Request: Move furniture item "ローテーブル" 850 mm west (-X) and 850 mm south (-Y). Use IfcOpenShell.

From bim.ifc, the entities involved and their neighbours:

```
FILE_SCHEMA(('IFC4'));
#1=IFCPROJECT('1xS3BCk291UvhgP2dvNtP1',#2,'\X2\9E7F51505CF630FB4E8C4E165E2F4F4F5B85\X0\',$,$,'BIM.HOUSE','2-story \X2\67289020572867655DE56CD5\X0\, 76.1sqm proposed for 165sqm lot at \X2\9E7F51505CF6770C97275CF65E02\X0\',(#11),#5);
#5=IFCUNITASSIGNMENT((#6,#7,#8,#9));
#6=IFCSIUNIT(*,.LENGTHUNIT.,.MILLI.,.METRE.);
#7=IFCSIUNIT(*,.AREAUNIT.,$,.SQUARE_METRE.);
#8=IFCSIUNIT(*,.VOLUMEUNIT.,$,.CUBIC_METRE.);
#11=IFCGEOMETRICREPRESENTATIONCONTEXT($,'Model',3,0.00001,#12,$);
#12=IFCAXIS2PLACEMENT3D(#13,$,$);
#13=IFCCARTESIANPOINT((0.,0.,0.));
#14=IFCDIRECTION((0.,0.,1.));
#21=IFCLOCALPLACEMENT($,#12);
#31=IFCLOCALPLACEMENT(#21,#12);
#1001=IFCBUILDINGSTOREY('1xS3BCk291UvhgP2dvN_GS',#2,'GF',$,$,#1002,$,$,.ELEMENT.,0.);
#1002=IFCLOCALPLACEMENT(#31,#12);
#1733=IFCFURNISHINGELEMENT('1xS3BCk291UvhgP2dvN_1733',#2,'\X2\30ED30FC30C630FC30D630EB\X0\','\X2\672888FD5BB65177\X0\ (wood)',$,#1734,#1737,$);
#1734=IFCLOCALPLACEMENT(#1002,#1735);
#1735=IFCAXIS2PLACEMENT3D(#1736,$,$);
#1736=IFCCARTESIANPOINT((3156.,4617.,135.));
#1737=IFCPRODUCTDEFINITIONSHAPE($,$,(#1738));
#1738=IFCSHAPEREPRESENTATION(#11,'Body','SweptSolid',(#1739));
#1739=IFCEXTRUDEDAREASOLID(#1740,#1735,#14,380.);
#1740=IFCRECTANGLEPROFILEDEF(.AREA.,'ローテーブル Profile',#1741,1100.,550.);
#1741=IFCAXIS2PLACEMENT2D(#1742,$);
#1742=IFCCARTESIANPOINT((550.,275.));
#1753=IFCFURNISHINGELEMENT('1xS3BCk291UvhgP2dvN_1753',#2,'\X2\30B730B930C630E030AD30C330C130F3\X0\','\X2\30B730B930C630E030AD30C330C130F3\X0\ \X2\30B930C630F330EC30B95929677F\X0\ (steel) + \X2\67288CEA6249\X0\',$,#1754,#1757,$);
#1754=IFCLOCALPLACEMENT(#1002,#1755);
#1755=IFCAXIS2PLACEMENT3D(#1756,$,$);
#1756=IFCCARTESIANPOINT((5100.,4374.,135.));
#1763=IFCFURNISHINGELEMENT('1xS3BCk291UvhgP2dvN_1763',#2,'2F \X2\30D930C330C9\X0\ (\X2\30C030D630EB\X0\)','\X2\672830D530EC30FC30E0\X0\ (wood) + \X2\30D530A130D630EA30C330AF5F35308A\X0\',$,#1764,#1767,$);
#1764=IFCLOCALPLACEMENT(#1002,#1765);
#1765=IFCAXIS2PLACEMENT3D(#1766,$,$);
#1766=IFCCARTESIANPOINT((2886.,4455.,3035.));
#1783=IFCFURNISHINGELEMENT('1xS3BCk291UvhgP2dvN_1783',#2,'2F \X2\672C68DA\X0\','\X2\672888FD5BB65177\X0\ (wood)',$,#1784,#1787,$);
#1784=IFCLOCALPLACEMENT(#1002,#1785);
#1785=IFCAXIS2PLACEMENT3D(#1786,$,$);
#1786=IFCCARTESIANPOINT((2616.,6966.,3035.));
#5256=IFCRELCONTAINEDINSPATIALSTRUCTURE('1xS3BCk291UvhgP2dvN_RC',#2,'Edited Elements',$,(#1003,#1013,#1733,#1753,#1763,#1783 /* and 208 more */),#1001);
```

```python
import ifcopenshell
import ifcopenshell.api.geometry
import ifcopenshell.util.placement
import ifcopenshell.util.unit

model = ifcopenshell.open("bim.ifc")
unit_scale = ifcopenshell.util.unit.calculate_unit_scale(model)

item = model.by_guid("1xS3BCk291UvhgP2dvN_1733")
matrix = ifcopenshell.util.placement.get_local_placement(item.ObjectPlacement)
matrix[0, 3] -= 0.85 / unit_scale
matrix[1, 3] -= 0.85 / unit_scale
ifcopenshell.api.geometry.edit_object_placement(model, product=item, matrix=matrix, is_si=False)

print(ifcopenshell.util.placement.get_local_placement(item.ObjectPlacement).round(3) + 0.0)

model.write("bim_rev.ifc")
```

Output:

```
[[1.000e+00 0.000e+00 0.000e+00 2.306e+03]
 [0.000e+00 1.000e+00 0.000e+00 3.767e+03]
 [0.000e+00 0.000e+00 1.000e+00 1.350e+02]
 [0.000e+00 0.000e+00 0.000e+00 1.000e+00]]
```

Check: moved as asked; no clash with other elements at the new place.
